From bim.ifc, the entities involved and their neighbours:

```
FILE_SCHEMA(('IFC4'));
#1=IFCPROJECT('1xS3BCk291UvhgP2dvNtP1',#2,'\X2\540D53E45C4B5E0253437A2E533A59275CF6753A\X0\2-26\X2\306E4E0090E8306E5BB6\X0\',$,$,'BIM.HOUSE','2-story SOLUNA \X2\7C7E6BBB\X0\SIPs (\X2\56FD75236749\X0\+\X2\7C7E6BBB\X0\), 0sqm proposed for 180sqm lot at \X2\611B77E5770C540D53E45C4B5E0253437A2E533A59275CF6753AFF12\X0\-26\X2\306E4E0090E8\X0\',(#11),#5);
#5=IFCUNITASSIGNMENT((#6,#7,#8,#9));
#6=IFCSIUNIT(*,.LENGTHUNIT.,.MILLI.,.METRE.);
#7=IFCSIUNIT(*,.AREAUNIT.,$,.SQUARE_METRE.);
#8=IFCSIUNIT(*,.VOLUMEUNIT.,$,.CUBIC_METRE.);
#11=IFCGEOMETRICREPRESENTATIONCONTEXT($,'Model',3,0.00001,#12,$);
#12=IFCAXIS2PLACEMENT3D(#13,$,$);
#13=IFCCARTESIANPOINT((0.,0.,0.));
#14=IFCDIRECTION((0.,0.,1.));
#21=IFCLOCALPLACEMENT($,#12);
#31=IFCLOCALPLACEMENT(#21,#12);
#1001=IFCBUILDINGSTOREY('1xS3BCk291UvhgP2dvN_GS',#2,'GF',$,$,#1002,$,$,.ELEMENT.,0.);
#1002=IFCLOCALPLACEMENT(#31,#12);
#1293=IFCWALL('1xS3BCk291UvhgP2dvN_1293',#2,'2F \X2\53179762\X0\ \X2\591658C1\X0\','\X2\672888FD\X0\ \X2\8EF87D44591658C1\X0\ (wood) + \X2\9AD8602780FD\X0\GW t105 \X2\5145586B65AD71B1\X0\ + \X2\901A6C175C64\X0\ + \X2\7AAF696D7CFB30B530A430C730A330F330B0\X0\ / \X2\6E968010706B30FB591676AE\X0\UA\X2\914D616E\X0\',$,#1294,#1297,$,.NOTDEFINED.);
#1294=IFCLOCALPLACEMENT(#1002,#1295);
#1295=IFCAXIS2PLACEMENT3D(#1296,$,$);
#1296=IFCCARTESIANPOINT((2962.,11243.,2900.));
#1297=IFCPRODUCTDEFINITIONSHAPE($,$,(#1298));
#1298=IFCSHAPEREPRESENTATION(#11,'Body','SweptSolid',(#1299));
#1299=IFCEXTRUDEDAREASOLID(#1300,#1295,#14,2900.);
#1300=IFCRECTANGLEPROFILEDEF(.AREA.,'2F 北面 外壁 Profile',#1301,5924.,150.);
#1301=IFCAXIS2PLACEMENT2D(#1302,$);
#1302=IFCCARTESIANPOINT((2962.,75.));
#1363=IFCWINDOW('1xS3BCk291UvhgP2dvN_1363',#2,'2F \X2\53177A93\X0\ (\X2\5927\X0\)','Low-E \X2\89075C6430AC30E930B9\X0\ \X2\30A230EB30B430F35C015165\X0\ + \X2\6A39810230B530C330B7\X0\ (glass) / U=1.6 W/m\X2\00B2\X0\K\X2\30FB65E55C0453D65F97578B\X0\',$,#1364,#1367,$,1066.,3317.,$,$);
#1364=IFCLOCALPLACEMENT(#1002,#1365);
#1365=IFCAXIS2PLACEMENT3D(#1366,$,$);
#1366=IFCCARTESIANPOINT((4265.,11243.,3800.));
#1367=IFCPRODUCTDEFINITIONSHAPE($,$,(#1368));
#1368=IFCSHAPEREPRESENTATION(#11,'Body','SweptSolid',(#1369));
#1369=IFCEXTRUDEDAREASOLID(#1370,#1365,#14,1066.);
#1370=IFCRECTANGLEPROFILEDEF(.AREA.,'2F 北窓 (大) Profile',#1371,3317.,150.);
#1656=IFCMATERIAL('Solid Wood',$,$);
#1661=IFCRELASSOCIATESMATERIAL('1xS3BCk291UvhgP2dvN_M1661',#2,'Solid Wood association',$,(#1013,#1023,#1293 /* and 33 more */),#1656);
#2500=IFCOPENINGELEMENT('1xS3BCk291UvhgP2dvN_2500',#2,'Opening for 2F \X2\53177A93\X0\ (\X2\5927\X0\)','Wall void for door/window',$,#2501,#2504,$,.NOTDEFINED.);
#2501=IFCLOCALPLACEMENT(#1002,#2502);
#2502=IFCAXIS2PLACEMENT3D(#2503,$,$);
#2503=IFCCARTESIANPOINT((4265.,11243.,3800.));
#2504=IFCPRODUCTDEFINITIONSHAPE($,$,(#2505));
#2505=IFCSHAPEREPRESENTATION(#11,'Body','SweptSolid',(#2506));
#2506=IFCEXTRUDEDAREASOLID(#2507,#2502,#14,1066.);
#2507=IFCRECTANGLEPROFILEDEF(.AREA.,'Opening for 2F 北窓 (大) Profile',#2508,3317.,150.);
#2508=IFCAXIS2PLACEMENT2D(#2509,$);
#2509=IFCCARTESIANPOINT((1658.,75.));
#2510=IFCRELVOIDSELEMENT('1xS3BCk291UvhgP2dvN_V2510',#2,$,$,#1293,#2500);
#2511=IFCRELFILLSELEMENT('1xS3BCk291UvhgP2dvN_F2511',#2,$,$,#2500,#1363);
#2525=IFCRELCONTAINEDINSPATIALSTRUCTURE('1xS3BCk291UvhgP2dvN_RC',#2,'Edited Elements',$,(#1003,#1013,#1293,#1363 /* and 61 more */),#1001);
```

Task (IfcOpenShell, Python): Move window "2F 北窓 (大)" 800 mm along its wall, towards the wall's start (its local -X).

```python
import ifcopenshell
import ifcopenshell.api.geometry
import ifcopenshell.util.placement
import ifcopenshell.util.unit

model = ifcopenshell.open("bim.ifc")
unit_scale = ifcopenshell.util.unit.calculate_unit_scale(model)

window = model.by_guid("1xS3BCk291UvhgP2dvN_1363")
opening = window.FillsVoids[0].RelatingOpeningElement
wall = opening.VoidsElements[0].RelatingBuildingElement

wall_matrix = ifcopenshell.util.placement.get_local_placement(wall.ObjectPlacement)
shift = wall_matrix[:3, 0] * -0.8 / unit_scale
before = ifcopenshell.util.placement.get_local_placement(window.ObjectPlacement)[:3, 3].copy()

# The window is not placed relative to its opening, so move both.
for product in (opening, window):
    matrix = ifcopenshell.util.placement.get_local_placement(product.ObjectPlacement)
    matrix[:3, 3] += shift
    ifcopenshell.api.geometry.edit_object_placement(model, product=product, matrix=matrix, is_si=False)

after = ifcopenshell.util.placement.get_local_placement(window.ObjectPlacement)[:3, 3]
print("window moved by", (after - before).round(3) + 0.0)

model.write("bim_updated.ifc")
```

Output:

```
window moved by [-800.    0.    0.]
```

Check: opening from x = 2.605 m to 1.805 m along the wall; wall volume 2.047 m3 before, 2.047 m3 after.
